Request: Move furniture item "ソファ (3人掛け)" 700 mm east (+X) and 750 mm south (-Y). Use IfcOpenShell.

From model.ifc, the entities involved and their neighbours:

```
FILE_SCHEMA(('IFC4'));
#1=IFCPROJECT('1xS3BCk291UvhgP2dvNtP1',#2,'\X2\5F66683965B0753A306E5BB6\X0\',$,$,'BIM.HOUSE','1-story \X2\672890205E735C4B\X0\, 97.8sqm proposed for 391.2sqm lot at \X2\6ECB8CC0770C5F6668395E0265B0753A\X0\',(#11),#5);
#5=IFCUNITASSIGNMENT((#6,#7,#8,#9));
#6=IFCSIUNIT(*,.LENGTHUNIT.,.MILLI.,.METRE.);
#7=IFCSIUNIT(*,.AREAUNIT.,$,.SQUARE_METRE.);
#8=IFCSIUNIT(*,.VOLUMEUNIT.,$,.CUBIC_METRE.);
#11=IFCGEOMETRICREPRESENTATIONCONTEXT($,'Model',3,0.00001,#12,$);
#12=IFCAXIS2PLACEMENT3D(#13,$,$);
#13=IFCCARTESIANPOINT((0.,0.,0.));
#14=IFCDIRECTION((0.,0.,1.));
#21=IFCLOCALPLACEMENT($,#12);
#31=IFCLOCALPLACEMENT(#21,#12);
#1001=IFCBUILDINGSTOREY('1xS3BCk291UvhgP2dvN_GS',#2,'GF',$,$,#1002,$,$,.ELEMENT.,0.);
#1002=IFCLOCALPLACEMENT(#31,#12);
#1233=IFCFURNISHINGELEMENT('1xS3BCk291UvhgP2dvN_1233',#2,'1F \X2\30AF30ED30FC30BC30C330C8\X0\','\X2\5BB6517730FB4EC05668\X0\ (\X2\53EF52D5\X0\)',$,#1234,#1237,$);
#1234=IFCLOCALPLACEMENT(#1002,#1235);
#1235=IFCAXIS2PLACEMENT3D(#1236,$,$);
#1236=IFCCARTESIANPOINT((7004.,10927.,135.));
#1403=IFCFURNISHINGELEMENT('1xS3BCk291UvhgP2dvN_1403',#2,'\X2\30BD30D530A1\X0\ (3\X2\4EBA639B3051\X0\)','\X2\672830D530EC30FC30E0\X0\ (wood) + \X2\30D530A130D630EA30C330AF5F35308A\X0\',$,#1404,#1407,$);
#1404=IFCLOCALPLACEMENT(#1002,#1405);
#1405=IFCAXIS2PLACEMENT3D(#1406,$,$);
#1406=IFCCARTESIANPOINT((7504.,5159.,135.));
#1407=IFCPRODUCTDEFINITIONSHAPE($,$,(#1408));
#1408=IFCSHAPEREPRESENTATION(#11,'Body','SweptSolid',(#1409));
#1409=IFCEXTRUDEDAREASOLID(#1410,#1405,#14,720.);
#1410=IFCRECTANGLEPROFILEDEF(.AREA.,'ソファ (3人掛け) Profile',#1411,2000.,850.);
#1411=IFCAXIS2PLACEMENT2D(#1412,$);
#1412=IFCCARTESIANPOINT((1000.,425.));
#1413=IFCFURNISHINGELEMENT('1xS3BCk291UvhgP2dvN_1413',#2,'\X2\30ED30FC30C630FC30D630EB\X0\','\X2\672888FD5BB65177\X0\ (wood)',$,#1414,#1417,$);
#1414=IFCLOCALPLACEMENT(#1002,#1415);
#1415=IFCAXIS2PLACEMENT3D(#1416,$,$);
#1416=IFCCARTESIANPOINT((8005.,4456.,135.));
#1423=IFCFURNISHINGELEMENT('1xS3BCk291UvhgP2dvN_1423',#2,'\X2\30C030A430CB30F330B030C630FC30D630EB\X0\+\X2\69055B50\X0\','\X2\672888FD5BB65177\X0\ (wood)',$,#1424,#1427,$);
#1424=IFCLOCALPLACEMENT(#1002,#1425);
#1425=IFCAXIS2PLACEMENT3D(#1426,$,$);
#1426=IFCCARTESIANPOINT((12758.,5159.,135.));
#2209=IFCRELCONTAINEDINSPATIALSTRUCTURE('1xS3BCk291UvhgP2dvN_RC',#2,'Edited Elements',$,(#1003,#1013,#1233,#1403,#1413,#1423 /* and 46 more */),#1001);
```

```python
import ifcopenshell
import ifcopenshell.api.geometry
import ifcopenshell.util.placement
import ifcopenshell.util.unit

model = ifcopenshell.open("model.ifc")
unit_scale = ifcopenshell.util.unit.calculate_unit_scale(model)

item = model.by_guid("1xS3BCk291UvhgP2dvN_1403")
matrix = ifcopenshell.util.placement.get_local_placement(item.ObjectPlacement)
matrix[0, 3] += 0.7 / unit_scale
matrix[1, 3] -= 0.75 / unit_scale
ifcopenshell.api.geometry.edit_object_placement(model, product=item, matrix=matrix, is_si=False)

print(ifcopenshell.util.placement.get_local_placement(item.ObjectPlacement).round(3) + 0.0)

model.write("model_v2.ifc")
```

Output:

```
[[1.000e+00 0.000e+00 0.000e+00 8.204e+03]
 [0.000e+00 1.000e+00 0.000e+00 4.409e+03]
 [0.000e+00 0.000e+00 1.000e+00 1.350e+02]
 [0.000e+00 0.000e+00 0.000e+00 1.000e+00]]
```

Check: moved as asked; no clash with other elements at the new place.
